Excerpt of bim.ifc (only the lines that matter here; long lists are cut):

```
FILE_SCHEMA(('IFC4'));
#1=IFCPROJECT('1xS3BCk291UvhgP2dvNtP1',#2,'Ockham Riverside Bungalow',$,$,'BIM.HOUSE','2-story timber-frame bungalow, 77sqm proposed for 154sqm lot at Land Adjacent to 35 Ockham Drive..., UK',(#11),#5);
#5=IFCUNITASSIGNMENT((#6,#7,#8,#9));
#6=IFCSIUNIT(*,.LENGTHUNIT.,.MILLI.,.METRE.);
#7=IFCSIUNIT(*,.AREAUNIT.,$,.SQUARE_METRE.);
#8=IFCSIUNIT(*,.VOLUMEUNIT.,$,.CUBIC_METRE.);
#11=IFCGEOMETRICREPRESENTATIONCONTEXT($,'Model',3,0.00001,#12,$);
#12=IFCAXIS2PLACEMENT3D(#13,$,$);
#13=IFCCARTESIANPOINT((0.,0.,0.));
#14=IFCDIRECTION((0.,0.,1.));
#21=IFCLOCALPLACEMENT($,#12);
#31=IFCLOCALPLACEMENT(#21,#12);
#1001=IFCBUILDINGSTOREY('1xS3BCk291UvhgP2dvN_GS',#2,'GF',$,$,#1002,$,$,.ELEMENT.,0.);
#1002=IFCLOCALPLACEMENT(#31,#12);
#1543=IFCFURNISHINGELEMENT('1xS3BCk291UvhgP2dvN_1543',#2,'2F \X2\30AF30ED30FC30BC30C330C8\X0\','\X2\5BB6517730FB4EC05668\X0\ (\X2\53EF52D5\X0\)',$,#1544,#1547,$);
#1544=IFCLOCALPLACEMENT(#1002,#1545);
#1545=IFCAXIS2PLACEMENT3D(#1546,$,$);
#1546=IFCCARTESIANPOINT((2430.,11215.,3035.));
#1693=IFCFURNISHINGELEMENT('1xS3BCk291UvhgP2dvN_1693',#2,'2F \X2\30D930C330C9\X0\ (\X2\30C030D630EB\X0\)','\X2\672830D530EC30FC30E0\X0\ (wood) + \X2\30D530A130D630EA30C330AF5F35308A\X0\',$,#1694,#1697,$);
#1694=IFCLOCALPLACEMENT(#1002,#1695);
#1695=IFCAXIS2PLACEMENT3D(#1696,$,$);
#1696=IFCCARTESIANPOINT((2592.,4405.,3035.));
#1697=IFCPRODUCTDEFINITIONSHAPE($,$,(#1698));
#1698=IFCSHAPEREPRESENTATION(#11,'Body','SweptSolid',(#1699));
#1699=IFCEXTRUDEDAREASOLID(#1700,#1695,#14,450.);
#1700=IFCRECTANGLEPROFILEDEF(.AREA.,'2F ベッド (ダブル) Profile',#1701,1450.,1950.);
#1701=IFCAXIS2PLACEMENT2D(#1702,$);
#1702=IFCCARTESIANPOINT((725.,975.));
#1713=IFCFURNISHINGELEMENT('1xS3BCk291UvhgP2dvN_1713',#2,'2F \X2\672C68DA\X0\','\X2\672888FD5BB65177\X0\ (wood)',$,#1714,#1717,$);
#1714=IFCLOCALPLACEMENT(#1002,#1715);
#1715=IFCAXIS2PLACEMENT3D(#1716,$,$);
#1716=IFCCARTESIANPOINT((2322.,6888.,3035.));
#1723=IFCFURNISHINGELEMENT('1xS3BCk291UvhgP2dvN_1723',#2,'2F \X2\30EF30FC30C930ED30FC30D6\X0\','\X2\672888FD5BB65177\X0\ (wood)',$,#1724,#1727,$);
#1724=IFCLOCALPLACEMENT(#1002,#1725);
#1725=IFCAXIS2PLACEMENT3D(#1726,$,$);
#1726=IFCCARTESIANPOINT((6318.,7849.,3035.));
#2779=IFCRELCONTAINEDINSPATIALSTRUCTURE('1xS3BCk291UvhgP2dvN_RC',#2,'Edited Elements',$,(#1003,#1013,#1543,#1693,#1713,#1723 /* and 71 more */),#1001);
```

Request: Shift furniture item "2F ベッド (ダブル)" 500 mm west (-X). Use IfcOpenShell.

```python
import ifcopenshell
import ifcopenshell.api.geometry
import ifcopenshell.util.placement
import ifcopenshell.util.unit

model = ifcopenshell.open("bim.ifc")
unit_scale = ifcopenshell.util.unit.calculate_unit_scale(model)

item = model.by_id(1693)
matrix = ifcopenshell.util.placement.get_local_placement(item.ObjectPlacement)
matrix[0, 3] -= 0.5 / unit_scale
ifcopenshell.api.geometry.edit_object_placement(model, product=item, matrix=matrix, is_si=False)

print(ifcopenshell.util.placement.get_local_placement(item.ObjectPlacement).round(3) + 0.0)

model.write("bim_rev.ifc")
```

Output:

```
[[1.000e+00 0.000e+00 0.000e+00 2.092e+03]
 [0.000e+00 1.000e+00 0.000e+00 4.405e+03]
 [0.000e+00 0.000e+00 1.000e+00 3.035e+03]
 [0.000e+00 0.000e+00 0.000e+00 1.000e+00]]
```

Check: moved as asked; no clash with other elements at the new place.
